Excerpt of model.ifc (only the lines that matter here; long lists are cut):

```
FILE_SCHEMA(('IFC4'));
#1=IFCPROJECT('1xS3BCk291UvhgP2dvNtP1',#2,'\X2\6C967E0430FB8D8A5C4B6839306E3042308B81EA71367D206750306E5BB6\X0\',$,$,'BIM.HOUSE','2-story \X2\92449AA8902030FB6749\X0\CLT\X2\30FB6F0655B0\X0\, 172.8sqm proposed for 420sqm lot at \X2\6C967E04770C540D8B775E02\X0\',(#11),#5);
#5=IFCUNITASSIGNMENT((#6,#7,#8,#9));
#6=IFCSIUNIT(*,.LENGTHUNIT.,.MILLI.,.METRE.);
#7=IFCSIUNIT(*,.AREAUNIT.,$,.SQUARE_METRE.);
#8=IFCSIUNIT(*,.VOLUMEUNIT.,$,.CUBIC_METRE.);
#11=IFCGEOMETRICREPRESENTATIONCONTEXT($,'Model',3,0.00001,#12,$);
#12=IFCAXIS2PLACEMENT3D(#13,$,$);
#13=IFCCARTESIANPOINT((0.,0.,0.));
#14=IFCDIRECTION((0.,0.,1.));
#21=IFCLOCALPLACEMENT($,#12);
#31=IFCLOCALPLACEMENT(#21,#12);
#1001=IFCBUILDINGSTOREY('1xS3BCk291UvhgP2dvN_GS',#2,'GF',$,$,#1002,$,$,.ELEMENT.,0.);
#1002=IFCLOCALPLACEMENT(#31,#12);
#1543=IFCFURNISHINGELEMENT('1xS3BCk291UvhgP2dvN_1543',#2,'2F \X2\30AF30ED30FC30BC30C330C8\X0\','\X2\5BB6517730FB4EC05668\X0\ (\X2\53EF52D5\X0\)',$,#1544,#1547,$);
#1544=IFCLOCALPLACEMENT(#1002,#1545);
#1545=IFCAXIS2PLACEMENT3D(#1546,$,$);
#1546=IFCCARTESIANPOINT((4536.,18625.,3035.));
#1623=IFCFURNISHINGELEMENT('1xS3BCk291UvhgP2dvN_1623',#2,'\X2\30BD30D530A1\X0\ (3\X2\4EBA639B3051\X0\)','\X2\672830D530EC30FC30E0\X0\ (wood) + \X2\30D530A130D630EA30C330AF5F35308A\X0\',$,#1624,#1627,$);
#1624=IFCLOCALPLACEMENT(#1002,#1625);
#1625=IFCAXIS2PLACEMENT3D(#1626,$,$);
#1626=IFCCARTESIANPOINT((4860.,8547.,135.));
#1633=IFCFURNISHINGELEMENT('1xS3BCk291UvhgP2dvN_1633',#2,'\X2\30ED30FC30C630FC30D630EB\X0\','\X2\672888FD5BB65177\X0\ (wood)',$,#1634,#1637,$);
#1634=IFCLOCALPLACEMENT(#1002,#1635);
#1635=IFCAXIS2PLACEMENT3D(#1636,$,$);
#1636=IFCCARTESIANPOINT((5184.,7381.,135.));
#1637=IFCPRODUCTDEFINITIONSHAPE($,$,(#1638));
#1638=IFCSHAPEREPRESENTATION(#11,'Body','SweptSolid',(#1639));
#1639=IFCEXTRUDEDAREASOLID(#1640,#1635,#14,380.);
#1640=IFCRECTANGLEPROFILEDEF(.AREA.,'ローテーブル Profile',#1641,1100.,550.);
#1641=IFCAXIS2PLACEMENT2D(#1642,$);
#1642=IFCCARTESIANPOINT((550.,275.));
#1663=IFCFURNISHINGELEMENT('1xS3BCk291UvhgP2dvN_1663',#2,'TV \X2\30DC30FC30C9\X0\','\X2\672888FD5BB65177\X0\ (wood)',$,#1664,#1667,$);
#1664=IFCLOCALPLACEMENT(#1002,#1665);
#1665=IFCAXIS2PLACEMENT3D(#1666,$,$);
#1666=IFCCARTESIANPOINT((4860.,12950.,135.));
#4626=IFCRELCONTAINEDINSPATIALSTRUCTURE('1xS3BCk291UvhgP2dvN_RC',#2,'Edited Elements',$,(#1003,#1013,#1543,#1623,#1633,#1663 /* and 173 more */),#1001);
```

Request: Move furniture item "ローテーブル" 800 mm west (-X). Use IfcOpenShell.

```python
import ifcopenshell
import ifcopenshell.api.geometry
import ifcopenshell.util.placement

model = ifcopenshell.open("model.ifc")

item = model.by_id(1633)
matrix = ifcopenshell.util.placement.get_local_placement(item.ObjectPlacement)
matrix[0, 3] -= 800.0
ifcopenshell.api.geometry.edit_object_placement(model, product=item, matrix=matrix, is_si=False)

print(ifcopenshell.util.placement.get_local_placement(item.ObjectPlacement).round(3) + 0.0)

model.write("model-out.ifc")
```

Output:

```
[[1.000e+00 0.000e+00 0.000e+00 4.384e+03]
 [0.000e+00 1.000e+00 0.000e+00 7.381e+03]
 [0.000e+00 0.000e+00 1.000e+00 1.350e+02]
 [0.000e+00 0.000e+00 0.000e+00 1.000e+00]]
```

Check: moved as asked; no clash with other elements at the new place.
